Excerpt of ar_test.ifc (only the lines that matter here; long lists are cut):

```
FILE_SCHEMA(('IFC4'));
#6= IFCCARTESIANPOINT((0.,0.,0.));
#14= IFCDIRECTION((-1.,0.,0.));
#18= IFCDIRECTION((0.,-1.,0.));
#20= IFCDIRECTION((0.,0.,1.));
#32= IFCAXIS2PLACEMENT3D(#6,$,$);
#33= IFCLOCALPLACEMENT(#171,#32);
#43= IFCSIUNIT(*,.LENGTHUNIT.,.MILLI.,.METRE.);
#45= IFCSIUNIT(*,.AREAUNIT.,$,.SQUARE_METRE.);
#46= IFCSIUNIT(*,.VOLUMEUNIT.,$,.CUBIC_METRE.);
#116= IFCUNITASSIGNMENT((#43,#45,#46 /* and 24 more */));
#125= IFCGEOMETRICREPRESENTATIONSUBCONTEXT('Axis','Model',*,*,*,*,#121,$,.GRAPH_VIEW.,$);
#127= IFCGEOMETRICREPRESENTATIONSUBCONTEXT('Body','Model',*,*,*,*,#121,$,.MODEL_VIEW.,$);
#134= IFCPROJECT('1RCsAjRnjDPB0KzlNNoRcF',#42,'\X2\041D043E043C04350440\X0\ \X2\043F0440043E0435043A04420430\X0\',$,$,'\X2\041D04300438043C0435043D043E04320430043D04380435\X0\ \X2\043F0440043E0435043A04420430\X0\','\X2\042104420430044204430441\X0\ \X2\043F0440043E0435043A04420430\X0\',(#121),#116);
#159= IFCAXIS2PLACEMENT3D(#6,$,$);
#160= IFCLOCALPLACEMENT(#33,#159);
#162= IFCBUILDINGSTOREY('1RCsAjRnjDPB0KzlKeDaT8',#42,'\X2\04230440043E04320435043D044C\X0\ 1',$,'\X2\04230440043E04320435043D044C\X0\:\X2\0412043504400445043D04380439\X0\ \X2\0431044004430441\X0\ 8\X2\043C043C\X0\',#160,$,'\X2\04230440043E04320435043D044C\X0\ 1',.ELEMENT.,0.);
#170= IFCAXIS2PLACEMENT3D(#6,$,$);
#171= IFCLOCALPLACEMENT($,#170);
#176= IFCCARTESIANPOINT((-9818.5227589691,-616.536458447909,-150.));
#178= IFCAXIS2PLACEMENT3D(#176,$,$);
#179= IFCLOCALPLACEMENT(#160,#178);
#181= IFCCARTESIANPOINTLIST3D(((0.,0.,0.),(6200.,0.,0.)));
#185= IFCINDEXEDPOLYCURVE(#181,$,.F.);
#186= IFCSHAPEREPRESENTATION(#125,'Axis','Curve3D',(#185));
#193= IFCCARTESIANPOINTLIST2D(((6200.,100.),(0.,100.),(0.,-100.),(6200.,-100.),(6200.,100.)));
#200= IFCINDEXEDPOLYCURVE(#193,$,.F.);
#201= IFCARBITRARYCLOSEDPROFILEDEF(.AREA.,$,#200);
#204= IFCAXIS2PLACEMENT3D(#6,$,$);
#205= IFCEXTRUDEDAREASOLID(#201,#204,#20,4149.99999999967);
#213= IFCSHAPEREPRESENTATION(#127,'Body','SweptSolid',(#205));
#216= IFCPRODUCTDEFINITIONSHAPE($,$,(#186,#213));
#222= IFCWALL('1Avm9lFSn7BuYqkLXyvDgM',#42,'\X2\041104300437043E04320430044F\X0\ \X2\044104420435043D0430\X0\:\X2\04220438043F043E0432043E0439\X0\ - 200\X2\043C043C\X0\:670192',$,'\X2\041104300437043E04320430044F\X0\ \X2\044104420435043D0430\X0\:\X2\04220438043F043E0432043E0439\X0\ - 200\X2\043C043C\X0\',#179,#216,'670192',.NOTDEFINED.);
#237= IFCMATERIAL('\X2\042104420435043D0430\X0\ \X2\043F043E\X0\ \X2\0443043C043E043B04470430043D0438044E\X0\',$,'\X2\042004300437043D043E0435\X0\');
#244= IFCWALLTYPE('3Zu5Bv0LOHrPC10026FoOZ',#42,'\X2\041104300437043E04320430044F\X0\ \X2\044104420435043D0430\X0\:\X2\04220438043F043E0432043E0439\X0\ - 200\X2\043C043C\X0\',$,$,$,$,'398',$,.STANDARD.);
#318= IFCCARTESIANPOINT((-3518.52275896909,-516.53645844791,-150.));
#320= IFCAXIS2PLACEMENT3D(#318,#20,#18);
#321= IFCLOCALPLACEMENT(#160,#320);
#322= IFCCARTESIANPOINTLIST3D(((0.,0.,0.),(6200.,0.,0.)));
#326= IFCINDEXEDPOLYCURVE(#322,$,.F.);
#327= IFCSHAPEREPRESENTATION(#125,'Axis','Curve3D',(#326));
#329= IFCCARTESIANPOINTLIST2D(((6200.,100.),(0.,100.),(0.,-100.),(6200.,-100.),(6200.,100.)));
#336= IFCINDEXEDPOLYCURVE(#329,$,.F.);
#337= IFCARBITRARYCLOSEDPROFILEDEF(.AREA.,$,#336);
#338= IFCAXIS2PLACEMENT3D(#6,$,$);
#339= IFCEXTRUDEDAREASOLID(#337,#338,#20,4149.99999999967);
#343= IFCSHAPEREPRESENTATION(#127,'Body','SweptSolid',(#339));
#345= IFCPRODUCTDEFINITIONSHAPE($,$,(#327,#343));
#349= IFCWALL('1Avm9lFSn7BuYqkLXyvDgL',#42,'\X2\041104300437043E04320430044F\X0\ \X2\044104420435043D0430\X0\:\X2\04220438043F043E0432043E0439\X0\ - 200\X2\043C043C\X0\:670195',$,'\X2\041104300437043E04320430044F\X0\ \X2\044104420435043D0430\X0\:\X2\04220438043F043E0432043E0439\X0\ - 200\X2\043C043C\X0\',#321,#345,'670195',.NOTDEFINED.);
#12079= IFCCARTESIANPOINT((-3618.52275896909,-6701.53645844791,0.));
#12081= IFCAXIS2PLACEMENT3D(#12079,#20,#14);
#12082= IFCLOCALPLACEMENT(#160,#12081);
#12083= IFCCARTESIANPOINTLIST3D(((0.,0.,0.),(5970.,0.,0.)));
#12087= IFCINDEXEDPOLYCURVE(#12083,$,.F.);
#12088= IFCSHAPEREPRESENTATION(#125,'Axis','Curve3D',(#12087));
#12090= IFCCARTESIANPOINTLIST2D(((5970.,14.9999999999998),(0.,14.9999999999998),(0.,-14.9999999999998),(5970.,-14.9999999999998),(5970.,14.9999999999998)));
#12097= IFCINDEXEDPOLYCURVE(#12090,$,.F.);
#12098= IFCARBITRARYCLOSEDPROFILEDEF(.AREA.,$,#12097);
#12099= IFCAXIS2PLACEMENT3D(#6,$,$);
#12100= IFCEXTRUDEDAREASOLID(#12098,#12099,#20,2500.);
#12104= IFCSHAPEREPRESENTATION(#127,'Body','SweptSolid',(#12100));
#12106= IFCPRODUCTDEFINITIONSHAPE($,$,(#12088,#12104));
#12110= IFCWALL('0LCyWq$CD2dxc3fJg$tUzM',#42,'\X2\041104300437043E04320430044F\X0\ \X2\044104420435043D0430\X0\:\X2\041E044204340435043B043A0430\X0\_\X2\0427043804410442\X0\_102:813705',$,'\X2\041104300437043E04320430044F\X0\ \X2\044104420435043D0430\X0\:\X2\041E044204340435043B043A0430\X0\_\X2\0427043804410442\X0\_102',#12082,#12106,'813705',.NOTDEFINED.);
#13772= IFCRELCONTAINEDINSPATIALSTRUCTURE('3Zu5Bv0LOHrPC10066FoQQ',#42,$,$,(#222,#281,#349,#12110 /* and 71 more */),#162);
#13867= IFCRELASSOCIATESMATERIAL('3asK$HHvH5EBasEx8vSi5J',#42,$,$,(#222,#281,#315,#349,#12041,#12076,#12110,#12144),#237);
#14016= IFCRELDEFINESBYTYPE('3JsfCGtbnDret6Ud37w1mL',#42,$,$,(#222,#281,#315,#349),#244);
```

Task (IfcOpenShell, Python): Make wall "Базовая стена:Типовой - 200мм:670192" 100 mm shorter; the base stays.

```python
import ifcopenshell
import ifcopenshell.geom
import ifcopenshell.util.representation
import ifcopenshell.util.shape

model = ifcopenshell.open("ar_test.ifc")
settings = ifcopenshell.geom.settings()


def volume(element):
    """Net volume in cubic metres, openings subtracted."""
    shape = ifcopenshell.geom.create_shape(settings, element)
    return ifcopenshell.util.shape.get_volume(shape.geometry)


wall = model.by_guid("1Avm9lFSn7BuYqkLXyvDgM")
before = volume(wall)

body = ifcopenshell.util.representation.get_representation(wall, "Model", "Body")
solid = body.Items[0]
old_height = solid.Depth
solid.Depth -= 100.0
after = volume(wall)

print(f"height {old_height:g} -> {solid.Depth:g}, volume {before:.3f} -> {after:.3f} m3")

model.write("ar_test_v2.ifc")
```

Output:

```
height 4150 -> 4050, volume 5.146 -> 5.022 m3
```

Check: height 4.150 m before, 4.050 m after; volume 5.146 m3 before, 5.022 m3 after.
